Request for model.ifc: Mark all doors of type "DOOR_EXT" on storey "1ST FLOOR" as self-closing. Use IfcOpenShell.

First a look at what the model holds.

```python
import ifcopenshell
import ifcopenshell.util.element

model = ifcopenshell.open("model.ifc")
print(model.schema)
storey = next(s for s in model.by_type("IfcBuildingStorey") if s.Name == "1ST FLOOR")
doors = [e for e in ifcopenshell.util.element.get_decomposition(storey) if e.is_a("IfcDoor")]
seen = {}
for e in doors:
    element_type = ifcopenshell.util.element.get_type(e)
    key = (element_type.Name if element_type != e and element_type else None, ifcopenshell.util.element.get_pset(e, "Pset_DoorCommon", "SelfClosing"))
    seen[key] = seen.get(key, 0) + 1
for (name, value), count in sorted(seen.items(), key=str):
    print(count, "x", name, "|", value)
```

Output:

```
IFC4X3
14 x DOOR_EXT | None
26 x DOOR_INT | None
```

```python
import ifcopenshell
import ifcopenshell.api.pset
import ifcopenshell.util.element

model = ifcopenshell.open("model.ifc")

storey = next(s for s in model.by_type("IfcBuildingStorey") if s.Name == "1ST FLOOR")
doors = [e for e in ifcopenshell.util.element.get_decomposition(storey) if e.is_a("IfcDoor")]

count = 0
for e in doors:
    element_type = ifcopenshell.util.element.get_type(e)
    if element_type in (None, e) or element_type.Name != "DOOR_EXT":
        continue
    # add_pset returns the element's existing set when there is one.
    pset = ifcopenshell.api.pset.add_pset(model, product=e, name="Pset_DoorCommon")
    ifcopenshell.api.pset.edit_pset(model, pset=pset, properties={"SelfClosing": True})
    count += 1

print(count, "doors updated")

model.write("model_updated.ifc")
```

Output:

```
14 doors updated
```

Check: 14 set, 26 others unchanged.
